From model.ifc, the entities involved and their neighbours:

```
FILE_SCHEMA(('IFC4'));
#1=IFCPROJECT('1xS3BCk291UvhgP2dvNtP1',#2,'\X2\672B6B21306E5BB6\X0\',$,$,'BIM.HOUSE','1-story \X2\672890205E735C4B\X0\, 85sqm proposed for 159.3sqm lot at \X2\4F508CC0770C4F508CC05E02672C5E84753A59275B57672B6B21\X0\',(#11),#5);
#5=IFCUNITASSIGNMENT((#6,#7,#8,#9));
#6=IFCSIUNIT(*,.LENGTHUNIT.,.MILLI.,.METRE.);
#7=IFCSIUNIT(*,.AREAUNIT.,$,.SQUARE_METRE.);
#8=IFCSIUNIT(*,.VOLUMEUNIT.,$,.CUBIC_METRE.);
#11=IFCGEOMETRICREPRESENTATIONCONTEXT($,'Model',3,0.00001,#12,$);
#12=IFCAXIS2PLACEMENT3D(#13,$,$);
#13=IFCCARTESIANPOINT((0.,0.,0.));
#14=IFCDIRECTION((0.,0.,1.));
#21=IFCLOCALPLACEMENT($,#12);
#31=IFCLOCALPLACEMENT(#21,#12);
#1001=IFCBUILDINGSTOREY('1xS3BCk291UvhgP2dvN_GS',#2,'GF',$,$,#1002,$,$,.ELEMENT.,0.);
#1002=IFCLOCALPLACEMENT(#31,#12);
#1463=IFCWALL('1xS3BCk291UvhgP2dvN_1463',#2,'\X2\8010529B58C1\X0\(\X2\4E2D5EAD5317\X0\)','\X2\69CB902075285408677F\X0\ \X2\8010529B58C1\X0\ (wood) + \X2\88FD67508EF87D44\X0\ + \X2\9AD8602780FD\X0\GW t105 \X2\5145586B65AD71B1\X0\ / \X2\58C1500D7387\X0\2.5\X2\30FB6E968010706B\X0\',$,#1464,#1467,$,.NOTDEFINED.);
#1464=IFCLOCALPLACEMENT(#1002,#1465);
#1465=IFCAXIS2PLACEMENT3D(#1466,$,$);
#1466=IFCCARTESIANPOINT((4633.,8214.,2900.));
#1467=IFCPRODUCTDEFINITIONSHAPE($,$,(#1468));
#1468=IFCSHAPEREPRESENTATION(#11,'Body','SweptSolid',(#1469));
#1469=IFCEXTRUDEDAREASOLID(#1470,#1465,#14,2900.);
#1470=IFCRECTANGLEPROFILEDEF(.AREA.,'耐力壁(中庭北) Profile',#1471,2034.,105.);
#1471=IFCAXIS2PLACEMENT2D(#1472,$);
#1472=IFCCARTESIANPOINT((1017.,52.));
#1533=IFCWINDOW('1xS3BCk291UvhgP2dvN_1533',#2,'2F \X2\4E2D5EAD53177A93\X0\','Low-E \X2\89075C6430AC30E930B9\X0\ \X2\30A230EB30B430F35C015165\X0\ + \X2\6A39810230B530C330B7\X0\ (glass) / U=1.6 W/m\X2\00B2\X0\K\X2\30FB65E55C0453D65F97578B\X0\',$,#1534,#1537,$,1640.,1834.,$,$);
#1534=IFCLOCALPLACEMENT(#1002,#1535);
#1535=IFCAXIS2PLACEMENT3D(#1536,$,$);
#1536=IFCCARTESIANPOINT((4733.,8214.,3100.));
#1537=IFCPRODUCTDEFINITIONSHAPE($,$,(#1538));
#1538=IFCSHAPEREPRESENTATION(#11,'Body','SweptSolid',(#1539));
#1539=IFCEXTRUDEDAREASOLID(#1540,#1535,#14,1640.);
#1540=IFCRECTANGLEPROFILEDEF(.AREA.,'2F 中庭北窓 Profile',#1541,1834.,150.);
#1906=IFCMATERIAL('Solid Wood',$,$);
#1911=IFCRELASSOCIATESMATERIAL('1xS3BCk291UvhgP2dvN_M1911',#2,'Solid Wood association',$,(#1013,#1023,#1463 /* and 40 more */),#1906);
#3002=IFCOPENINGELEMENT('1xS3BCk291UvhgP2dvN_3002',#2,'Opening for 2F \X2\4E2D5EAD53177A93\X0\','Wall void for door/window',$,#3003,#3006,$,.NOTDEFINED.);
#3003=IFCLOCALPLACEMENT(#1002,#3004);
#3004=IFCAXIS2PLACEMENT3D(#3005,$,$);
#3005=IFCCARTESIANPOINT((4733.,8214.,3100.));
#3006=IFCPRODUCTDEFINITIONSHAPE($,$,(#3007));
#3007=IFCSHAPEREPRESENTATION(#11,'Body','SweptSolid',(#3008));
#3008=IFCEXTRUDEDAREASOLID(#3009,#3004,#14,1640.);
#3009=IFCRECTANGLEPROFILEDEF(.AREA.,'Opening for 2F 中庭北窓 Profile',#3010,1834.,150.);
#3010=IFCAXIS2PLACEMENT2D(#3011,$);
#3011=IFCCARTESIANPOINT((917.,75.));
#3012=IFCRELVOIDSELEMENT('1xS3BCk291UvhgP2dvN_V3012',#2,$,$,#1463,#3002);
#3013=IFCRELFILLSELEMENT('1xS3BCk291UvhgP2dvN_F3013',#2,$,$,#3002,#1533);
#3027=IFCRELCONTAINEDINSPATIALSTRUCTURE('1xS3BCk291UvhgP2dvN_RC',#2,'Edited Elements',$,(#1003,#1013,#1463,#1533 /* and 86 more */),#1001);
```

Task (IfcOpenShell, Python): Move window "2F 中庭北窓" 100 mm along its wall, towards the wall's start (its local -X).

```python
import ifcopenshell
import ifcopenshell.api.geometry
import ifcopenshell.util.placement

model = ifcopenshell.open("model.ifc")

window = model.by_id(1533)
opening = window.FillsVoids[0].RelatingOpeningElement
wall = opening.VoidsElements[0].RelatingBuildingElement

wall_matrix = ifcopenshell.util.placement.get_local_placement(wall.ObjectPlacement)
shift = wall_matrix[:3, 0] * -100.0
before = ifcopenshell.util.placement.get_local_placement(window.ObjectPlacement)[:3, 3].copy()

# The window is not placed relative to its opening, so move both.
for product in (opening, window):
    matrix = ifcopenshell.util.placement.get_local_placement(product.ObjectPlacement)
    matrix[:3, 3] += shift
    ifcopenshell.api.geometry.edit_object_placement(model, product=product, matrix=matrix, is_si=False)

after = ifcopenshell.util.placement.get_local_placement(window.ObjectPlacement)[:3, 3]
print("window moved by", (after - before).round(3) + 0.0)

model.write("model-out.ifc")
```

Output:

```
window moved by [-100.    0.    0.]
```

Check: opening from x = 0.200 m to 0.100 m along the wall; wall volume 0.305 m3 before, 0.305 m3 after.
